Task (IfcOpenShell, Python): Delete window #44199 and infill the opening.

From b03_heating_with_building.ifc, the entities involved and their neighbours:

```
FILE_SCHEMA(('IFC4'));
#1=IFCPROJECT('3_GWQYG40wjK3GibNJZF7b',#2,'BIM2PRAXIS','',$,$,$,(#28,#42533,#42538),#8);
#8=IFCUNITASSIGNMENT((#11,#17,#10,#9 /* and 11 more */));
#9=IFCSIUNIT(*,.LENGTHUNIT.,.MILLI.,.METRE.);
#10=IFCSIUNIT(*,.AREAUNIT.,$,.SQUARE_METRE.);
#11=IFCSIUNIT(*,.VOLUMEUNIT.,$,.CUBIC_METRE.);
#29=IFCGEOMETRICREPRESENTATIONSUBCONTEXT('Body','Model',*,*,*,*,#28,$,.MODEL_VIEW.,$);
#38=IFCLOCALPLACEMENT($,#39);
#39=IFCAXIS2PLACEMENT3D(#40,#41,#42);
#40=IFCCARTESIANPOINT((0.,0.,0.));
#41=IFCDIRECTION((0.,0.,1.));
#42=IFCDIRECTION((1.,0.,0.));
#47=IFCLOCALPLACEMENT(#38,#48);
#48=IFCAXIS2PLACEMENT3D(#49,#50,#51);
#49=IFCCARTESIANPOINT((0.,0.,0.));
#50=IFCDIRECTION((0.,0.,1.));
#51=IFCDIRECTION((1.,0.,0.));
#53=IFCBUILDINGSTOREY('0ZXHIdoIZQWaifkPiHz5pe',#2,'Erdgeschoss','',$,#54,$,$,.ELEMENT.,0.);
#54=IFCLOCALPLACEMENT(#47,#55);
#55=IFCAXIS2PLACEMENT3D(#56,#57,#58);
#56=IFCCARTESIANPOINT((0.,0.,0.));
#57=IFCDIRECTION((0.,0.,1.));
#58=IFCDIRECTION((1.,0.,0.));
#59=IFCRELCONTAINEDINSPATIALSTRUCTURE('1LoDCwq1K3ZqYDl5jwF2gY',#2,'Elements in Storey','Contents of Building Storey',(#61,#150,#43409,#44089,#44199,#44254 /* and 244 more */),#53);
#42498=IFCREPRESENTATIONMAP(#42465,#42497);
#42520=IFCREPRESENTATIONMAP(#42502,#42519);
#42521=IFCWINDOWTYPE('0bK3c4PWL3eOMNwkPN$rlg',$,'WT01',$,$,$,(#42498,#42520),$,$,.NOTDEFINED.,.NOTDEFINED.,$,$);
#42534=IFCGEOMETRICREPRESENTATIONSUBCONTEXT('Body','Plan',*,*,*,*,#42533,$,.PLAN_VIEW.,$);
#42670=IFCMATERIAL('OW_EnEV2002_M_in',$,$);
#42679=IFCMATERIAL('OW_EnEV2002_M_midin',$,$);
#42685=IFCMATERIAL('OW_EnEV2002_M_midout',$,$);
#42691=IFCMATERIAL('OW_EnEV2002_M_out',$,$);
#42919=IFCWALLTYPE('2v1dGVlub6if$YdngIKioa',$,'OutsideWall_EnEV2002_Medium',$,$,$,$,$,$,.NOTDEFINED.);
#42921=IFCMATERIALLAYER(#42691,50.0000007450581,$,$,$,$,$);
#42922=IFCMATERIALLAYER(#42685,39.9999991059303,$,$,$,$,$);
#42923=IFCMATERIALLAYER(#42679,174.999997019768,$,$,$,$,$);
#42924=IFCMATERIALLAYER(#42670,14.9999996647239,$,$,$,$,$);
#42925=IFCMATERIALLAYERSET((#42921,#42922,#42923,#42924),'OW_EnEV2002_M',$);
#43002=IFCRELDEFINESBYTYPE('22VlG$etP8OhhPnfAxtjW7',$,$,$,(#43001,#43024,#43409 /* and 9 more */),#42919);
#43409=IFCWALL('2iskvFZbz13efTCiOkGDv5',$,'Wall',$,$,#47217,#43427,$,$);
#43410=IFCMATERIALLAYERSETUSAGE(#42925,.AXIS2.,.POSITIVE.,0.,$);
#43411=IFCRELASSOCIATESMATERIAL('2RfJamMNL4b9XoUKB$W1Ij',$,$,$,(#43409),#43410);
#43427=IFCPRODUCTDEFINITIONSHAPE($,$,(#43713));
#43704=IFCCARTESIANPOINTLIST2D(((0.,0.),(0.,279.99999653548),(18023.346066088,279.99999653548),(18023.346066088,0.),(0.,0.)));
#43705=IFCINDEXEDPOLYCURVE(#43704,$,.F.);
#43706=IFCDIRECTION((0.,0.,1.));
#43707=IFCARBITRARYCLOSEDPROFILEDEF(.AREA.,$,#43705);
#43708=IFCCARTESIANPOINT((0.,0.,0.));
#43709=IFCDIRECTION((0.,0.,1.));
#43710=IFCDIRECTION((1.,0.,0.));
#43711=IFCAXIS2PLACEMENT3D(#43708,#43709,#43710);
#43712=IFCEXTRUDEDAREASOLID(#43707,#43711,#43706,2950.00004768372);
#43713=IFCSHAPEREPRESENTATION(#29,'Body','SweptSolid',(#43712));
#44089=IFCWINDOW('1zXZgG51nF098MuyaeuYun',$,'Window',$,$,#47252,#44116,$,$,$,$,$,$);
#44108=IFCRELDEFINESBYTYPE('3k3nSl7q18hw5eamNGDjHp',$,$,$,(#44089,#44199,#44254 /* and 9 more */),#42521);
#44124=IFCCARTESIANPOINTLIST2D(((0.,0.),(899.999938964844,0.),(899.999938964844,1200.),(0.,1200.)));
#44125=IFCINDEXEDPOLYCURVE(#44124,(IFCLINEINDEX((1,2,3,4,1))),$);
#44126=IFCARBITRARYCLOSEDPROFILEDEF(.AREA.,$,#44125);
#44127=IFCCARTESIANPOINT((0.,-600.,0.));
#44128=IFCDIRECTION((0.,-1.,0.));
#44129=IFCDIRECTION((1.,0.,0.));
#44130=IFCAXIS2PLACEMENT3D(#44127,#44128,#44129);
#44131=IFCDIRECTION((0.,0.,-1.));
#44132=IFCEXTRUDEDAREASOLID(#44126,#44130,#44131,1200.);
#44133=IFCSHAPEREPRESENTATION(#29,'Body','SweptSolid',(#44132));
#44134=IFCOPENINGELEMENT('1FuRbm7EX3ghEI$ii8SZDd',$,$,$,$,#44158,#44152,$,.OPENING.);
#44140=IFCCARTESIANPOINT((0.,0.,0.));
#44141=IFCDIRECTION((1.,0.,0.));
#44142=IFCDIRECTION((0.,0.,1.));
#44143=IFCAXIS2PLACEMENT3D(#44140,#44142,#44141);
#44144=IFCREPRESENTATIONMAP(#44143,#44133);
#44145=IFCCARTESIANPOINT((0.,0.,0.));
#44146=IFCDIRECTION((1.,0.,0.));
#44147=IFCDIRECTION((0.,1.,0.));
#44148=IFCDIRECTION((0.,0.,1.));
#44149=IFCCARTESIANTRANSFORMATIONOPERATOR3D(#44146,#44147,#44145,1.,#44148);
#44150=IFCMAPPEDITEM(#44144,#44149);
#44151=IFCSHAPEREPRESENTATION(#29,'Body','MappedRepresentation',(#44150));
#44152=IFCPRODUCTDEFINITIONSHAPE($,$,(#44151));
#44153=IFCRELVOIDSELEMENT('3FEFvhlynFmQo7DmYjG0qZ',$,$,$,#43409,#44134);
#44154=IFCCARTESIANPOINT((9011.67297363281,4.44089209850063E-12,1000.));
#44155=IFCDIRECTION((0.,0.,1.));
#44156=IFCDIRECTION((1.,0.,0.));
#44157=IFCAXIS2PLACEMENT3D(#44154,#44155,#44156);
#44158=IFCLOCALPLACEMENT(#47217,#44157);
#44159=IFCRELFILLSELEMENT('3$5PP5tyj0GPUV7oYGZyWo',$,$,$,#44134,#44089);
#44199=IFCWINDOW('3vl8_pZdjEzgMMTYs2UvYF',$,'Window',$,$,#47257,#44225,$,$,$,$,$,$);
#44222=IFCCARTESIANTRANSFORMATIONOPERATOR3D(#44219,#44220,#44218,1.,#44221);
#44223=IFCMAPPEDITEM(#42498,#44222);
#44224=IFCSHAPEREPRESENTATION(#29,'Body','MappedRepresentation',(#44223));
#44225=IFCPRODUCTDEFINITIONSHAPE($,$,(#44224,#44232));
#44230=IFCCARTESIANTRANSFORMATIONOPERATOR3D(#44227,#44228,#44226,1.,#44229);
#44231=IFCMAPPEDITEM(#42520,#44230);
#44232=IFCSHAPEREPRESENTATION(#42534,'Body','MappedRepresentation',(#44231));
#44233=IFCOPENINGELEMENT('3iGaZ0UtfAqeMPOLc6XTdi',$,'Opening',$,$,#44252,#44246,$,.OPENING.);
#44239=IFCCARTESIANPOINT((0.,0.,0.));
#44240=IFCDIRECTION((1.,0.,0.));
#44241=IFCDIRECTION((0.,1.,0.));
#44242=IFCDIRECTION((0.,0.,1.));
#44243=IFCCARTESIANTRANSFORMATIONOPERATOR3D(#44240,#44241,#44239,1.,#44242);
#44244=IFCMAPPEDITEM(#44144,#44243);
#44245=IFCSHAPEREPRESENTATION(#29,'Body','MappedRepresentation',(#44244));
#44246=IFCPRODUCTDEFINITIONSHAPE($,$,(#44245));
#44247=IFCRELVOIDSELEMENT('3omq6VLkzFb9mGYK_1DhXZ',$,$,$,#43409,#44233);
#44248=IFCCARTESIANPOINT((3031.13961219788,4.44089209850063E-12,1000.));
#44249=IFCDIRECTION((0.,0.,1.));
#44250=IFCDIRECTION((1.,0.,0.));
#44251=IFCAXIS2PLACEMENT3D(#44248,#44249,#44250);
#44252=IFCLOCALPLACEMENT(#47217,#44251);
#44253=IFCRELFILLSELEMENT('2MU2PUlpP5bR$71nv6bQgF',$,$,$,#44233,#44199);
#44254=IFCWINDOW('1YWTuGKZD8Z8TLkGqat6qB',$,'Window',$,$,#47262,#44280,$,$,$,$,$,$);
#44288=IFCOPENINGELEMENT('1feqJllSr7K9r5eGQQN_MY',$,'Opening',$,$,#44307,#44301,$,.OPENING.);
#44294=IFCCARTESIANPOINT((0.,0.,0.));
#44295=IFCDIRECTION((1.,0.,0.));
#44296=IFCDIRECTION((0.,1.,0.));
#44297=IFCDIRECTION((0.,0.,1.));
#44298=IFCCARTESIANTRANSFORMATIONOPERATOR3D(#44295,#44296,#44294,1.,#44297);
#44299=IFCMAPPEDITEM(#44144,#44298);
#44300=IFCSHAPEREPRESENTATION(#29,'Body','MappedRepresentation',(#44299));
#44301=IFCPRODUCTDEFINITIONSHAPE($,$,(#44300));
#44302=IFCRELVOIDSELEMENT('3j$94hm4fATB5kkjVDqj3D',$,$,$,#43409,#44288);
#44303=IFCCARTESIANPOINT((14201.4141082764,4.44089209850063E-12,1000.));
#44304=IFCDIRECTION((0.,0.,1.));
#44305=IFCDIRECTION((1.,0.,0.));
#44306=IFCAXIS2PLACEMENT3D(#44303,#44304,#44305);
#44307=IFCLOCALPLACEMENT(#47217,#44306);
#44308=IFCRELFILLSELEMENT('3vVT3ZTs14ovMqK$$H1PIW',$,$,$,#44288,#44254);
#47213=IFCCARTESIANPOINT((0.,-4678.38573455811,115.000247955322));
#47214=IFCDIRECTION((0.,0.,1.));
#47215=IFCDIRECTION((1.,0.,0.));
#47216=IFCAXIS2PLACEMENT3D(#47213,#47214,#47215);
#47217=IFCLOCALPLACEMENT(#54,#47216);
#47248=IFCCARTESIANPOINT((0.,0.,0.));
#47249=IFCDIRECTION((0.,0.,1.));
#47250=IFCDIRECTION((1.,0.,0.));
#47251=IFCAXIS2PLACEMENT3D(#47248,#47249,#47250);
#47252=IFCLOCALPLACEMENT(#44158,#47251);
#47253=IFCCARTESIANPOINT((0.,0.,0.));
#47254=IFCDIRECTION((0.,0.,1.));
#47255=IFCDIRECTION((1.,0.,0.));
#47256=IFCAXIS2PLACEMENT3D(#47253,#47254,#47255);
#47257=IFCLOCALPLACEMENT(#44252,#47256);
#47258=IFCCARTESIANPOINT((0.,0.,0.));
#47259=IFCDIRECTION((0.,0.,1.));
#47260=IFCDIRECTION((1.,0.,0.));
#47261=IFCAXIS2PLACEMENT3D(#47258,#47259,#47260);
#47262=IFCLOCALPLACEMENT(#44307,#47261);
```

```python
import ifcopenshell
import ifcopenshell.api.feature
import ifcopenshell.api.root
import ifcopenshell.geom
import ifcopenshell.util.shape

model = ifcopenshell.open("b03_heating_with_building.ifc")
settings = ifcopenshell.geom.settings()


def volume(element):
    """Net volume in cubic metres, openings subtracted."""
    shape = ifcopenshell.geom.create_shape(settings, element)
    return ifcopenshell.util.shape.get_volume(shape.geometry)


window = model.by_id(44199)
opening = window.FillsVoids[0].RelatingOpeningElement
wall = opening.VoidsElements[0].RelatingBuildingElement
before = volume(wall)

ifcopenshell.api.root.remove_product(model, product=window)
ifcopenshell.api.feature.remove_feature(model, feature=opening)

after = volume(wall)

print(f"wall volume {before:.3f} -> {after:.3f} m3")

model.write("b03_heating_with_building-out.ifc")
```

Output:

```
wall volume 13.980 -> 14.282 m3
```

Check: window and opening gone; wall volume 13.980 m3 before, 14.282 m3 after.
